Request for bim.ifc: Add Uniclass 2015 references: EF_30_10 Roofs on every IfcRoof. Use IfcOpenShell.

First a look at what the model holds.

```python
import ifcopenshell

model = ifcopenshell.open("bim.ifc")
print(model.schema)
print("classifications:", [c.Name for c in model.by_type("IfcClassification")])
for ifc_class in ("IfcDoor", "IfcRoof", "IfcStair", "IfcWall", "IfcWindow"):
    print(ifc_class, len(model.by_type(ifc_class)))
```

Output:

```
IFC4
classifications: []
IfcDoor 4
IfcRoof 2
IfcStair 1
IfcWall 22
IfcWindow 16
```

```python
import ifcopenshell
import ifcopenshell.api.classification

model = ifcopenshell.open("bim.ifc")

system = ifcopenshell.api.classification.add_classification(model, classification="Uniclass 2015")

codes = {
    "IfcRoof": ("EF_30_10", "Roofs"),
}
for ifc_class, (code, name) in codes.items():
    products = model.by_type(ifc_class)
    ifcopenshell.api.classification.add_reference(
        model, products=products, classification=system, identification=code, name=name
    )
    print(code, len(products))

model.write("bim-out.ifc")
```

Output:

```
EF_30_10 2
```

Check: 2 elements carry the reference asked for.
